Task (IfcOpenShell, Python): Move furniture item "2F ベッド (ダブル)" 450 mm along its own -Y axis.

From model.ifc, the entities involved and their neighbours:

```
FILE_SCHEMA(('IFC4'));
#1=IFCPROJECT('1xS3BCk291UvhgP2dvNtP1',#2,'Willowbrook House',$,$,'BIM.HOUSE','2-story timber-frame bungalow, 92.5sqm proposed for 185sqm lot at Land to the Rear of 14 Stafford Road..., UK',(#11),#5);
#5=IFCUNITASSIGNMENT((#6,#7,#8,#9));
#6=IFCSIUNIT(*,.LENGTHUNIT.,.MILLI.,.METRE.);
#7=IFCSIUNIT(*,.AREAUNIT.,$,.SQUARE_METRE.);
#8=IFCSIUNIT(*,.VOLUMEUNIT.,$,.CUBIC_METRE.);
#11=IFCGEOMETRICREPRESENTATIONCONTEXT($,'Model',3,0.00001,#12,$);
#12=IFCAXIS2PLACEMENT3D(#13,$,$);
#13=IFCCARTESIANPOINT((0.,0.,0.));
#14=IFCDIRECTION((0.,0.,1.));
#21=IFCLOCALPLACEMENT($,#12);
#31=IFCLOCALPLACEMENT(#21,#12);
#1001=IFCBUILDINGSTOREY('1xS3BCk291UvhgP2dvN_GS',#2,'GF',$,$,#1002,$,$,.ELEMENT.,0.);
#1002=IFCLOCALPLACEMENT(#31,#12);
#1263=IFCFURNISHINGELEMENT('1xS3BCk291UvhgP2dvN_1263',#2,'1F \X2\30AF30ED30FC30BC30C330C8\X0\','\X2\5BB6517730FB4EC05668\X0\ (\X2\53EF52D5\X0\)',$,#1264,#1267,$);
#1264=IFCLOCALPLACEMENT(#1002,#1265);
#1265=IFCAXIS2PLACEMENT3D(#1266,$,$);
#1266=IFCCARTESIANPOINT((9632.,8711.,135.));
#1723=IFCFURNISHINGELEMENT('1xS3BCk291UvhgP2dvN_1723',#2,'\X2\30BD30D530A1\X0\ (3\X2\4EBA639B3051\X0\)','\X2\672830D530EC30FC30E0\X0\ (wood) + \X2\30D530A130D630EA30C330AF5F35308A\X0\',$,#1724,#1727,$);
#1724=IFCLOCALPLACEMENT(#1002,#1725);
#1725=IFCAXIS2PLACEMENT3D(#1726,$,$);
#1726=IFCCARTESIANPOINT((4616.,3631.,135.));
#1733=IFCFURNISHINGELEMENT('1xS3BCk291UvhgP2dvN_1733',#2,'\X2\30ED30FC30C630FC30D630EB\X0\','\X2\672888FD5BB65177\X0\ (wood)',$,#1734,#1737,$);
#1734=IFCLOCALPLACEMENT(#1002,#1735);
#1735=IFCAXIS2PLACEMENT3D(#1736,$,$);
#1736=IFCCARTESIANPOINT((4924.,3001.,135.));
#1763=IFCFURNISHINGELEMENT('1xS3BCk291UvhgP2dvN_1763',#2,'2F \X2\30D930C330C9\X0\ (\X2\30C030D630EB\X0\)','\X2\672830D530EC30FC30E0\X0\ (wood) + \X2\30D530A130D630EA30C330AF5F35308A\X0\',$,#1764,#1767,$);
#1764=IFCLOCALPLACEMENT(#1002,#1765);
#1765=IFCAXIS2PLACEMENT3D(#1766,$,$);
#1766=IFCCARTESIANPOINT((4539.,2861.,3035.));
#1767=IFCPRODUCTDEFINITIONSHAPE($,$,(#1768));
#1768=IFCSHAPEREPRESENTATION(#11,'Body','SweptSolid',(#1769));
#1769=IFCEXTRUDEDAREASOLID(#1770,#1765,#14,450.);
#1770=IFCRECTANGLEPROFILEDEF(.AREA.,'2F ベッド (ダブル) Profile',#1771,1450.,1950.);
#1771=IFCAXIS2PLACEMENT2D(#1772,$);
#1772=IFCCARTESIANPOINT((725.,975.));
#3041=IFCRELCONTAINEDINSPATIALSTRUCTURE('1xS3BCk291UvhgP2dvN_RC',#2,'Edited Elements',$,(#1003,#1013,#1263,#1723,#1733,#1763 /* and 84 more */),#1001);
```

```python
import ifcopenshell
import ifcopenshell.api.geometry
import ifcopenshell.util.placement

model = ifcopenshell.open("model.ifc")

item = model.by_guid("1xS3BCk291UvhgP2dvN_1763")
matrix = ifcopenshell.util.placement.get_local_placement(item.ObjectPlacement)
matrix[:3, 3] -= matrix[:3, 1] * 450.0
ifcopenshell.api.geometry.edit_object_placement(model, product=item, matrix=matrix, is_si=False)

print(ifcopenshell.util.placement.get_local_placement(item.ObjectPlacement).round(3) + 0.0)

model.write("model-out.ifc")
```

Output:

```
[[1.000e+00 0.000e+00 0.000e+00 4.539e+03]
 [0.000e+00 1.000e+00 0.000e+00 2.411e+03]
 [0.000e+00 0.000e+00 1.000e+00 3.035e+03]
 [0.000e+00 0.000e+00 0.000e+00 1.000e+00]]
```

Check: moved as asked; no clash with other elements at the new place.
